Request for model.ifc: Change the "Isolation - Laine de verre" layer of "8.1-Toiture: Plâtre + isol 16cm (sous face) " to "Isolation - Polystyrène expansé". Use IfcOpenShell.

First a look at what the model holds.

```python
import ifcopenshell
import ifcopenshell.util.element

model = ifcopenshell.open("model.ifc")
print(model.schema)
for layer_set in model.by_type("IfcMaterialLayerSet"):
    if layer_set.LayerSetName == "8.1-Toiture: Plâtre + isol 16cm (sous face) ":
        for layer in layer_set.MaterialLayers:
            print(layer.id(), layer.Material and layer.Material.Name, layer.LayerThickness, sep=" | ")
        print(len(ifcopenshell.util.element.get_elements_by_material(model, layer_set)), "elements and types use it")
print(sorted(m.Name for m in model.by_type("IfcMaterial") if m.Name)[:60])
```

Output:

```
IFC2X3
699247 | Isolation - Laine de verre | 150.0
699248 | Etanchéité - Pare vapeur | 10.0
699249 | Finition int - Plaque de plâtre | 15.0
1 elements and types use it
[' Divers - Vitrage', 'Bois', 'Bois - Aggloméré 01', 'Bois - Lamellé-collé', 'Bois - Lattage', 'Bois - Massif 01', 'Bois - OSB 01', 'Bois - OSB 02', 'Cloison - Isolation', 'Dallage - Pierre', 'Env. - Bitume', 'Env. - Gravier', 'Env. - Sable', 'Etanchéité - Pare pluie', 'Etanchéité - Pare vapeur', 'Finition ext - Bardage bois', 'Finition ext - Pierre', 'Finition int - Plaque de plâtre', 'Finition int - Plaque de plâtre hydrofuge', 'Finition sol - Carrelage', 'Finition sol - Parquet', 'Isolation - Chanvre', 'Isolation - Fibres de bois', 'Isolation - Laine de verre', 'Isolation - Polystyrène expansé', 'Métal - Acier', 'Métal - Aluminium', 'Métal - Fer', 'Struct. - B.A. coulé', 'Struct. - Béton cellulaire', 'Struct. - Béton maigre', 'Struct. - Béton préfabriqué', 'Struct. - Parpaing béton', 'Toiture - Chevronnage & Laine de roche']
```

```python
import ifcopenshell
import ifcopenshell.api.material

model = ifcopenshell.open("model.ifc")

layer_set = next(s for s in model.by_type("IfcMaterialLayerSet") if s.LayerSetName == "8.1-Toiture: Plâtre + isol 16cm (sous face) ")
layer = next(l for l in layer_set.MaterialLayers if l.Material and l.Material.Name == "Isolation - Laine de verre")
material = next(m for m in model.by_type("IfcMaterial") if m.Name == "Isolation - Polystyrène expansé")

# Point this one layer at the other material; renaming the old one would change it everywhere.
ifcopenshell.api.material.edit_layer(model, layer=layer, attributes={}, material=material)

print([l.Material.Name if l.Material else None for l in layer_set.MaterialLayers])

model.write("model_rev.ifc")
```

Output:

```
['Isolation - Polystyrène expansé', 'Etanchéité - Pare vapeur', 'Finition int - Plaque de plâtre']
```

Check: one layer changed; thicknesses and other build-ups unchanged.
